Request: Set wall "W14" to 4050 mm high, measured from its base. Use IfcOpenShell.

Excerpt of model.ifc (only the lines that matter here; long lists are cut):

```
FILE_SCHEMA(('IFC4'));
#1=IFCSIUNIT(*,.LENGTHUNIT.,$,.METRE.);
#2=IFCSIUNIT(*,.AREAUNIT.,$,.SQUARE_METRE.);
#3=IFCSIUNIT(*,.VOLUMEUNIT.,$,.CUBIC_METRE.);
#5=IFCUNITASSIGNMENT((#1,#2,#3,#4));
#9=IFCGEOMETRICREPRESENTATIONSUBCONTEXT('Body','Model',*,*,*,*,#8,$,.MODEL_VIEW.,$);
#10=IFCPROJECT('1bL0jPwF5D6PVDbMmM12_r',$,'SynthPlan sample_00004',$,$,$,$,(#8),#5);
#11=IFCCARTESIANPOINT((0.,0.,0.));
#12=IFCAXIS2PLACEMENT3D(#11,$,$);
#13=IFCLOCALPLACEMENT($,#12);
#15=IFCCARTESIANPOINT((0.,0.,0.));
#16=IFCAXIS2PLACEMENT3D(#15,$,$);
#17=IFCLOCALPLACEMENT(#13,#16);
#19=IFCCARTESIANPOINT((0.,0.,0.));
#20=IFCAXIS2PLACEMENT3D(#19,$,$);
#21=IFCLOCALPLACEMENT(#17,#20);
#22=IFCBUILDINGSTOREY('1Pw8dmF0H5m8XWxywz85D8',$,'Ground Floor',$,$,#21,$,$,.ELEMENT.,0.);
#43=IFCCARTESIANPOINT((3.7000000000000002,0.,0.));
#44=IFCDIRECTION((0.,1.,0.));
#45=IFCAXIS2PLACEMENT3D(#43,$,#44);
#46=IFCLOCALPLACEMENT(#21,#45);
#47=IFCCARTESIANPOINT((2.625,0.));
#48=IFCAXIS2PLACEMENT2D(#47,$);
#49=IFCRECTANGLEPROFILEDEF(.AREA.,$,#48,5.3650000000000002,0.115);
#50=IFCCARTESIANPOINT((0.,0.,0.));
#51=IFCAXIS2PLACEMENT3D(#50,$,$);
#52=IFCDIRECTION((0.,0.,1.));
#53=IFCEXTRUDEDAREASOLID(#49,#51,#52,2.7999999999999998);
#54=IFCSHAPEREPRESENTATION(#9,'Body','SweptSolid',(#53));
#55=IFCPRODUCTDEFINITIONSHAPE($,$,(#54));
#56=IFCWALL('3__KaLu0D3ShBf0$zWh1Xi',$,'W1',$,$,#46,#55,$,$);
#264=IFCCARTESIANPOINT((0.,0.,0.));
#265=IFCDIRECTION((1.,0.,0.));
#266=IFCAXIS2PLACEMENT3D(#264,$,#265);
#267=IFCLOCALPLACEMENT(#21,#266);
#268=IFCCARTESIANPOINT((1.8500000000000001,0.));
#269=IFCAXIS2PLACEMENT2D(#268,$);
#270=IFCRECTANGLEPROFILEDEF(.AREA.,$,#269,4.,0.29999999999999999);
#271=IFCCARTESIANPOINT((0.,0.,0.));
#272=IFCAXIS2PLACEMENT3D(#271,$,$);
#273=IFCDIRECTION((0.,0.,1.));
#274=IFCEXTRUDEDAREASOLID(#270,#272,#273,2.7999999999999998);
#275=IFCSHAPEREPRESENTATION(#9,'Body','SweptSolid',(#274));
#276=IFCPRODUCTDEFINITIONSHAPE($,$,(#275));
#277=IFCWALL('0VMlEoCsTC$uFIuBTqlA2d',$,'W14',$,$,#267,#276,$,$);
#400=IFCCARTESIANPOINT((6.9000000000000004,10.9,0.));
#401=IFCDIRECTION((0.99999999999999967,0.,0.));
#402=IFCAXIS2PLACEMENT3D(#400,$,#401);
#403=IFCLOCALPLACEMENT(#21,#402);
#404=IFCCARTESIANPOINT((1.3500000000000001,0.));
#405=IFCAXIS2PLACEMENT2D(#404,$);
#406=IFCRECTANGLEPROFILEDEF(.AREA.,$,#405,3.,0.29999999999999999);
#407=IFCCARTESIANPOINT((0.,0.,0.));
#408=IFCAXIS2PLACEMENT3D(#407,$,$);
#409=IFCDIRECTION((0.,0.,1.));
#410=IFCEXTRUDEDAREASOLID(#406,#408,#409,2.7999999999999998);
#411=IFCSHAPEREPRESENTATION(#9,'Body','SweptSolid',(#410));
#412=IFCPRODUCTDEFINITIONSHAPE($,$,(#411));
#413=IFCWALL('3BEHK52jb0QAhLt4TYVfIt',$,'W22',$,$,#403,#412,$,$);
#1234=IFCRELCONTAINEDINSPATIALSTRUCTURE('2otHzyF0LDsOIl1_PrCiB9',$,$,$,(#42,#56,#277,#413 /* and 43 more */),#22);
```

```python
import ifcopenshell
import ifcopenshell.geom
import ifcopenshell.util.representation
import ifcopenshell.util.shape
import ifcopenshell.util.unit

model = ifcopenshell.open("model.ifc")
unit_scale = ifcopenshell.util.unit.calculate_unit_scale(model)
settings = ifcopenshell.geom.settings()


def volume(element):
    """Net volume in cubic metres, openings subtracted."""
    shape = ifcopenshell.geom.create_shape(settings, element)
    return ifcopenshell.util.shape.get_volume(shape.geometry)


wall = model.by_guid("0VMlEoCsTC$uFIuBTqlA2d")
before = volume(wall)

body = ifcopenshell.util.representation.get_representation(wall, "Model", "Body")
solid = body.Items[0]
old_height = solid.Depth
solid.Depth = 4.05 / unit_scale
after = volume(wall)

print(f"height {old_height:g} -> {solid.Depth:g}, volume {before:.3f} -> {after:.3f} m3")

model.write("model-out.ifc")
```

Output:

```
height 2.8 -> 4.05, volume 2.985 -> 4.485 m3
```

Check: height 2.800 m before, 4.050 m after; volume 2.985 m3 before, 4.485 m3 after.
